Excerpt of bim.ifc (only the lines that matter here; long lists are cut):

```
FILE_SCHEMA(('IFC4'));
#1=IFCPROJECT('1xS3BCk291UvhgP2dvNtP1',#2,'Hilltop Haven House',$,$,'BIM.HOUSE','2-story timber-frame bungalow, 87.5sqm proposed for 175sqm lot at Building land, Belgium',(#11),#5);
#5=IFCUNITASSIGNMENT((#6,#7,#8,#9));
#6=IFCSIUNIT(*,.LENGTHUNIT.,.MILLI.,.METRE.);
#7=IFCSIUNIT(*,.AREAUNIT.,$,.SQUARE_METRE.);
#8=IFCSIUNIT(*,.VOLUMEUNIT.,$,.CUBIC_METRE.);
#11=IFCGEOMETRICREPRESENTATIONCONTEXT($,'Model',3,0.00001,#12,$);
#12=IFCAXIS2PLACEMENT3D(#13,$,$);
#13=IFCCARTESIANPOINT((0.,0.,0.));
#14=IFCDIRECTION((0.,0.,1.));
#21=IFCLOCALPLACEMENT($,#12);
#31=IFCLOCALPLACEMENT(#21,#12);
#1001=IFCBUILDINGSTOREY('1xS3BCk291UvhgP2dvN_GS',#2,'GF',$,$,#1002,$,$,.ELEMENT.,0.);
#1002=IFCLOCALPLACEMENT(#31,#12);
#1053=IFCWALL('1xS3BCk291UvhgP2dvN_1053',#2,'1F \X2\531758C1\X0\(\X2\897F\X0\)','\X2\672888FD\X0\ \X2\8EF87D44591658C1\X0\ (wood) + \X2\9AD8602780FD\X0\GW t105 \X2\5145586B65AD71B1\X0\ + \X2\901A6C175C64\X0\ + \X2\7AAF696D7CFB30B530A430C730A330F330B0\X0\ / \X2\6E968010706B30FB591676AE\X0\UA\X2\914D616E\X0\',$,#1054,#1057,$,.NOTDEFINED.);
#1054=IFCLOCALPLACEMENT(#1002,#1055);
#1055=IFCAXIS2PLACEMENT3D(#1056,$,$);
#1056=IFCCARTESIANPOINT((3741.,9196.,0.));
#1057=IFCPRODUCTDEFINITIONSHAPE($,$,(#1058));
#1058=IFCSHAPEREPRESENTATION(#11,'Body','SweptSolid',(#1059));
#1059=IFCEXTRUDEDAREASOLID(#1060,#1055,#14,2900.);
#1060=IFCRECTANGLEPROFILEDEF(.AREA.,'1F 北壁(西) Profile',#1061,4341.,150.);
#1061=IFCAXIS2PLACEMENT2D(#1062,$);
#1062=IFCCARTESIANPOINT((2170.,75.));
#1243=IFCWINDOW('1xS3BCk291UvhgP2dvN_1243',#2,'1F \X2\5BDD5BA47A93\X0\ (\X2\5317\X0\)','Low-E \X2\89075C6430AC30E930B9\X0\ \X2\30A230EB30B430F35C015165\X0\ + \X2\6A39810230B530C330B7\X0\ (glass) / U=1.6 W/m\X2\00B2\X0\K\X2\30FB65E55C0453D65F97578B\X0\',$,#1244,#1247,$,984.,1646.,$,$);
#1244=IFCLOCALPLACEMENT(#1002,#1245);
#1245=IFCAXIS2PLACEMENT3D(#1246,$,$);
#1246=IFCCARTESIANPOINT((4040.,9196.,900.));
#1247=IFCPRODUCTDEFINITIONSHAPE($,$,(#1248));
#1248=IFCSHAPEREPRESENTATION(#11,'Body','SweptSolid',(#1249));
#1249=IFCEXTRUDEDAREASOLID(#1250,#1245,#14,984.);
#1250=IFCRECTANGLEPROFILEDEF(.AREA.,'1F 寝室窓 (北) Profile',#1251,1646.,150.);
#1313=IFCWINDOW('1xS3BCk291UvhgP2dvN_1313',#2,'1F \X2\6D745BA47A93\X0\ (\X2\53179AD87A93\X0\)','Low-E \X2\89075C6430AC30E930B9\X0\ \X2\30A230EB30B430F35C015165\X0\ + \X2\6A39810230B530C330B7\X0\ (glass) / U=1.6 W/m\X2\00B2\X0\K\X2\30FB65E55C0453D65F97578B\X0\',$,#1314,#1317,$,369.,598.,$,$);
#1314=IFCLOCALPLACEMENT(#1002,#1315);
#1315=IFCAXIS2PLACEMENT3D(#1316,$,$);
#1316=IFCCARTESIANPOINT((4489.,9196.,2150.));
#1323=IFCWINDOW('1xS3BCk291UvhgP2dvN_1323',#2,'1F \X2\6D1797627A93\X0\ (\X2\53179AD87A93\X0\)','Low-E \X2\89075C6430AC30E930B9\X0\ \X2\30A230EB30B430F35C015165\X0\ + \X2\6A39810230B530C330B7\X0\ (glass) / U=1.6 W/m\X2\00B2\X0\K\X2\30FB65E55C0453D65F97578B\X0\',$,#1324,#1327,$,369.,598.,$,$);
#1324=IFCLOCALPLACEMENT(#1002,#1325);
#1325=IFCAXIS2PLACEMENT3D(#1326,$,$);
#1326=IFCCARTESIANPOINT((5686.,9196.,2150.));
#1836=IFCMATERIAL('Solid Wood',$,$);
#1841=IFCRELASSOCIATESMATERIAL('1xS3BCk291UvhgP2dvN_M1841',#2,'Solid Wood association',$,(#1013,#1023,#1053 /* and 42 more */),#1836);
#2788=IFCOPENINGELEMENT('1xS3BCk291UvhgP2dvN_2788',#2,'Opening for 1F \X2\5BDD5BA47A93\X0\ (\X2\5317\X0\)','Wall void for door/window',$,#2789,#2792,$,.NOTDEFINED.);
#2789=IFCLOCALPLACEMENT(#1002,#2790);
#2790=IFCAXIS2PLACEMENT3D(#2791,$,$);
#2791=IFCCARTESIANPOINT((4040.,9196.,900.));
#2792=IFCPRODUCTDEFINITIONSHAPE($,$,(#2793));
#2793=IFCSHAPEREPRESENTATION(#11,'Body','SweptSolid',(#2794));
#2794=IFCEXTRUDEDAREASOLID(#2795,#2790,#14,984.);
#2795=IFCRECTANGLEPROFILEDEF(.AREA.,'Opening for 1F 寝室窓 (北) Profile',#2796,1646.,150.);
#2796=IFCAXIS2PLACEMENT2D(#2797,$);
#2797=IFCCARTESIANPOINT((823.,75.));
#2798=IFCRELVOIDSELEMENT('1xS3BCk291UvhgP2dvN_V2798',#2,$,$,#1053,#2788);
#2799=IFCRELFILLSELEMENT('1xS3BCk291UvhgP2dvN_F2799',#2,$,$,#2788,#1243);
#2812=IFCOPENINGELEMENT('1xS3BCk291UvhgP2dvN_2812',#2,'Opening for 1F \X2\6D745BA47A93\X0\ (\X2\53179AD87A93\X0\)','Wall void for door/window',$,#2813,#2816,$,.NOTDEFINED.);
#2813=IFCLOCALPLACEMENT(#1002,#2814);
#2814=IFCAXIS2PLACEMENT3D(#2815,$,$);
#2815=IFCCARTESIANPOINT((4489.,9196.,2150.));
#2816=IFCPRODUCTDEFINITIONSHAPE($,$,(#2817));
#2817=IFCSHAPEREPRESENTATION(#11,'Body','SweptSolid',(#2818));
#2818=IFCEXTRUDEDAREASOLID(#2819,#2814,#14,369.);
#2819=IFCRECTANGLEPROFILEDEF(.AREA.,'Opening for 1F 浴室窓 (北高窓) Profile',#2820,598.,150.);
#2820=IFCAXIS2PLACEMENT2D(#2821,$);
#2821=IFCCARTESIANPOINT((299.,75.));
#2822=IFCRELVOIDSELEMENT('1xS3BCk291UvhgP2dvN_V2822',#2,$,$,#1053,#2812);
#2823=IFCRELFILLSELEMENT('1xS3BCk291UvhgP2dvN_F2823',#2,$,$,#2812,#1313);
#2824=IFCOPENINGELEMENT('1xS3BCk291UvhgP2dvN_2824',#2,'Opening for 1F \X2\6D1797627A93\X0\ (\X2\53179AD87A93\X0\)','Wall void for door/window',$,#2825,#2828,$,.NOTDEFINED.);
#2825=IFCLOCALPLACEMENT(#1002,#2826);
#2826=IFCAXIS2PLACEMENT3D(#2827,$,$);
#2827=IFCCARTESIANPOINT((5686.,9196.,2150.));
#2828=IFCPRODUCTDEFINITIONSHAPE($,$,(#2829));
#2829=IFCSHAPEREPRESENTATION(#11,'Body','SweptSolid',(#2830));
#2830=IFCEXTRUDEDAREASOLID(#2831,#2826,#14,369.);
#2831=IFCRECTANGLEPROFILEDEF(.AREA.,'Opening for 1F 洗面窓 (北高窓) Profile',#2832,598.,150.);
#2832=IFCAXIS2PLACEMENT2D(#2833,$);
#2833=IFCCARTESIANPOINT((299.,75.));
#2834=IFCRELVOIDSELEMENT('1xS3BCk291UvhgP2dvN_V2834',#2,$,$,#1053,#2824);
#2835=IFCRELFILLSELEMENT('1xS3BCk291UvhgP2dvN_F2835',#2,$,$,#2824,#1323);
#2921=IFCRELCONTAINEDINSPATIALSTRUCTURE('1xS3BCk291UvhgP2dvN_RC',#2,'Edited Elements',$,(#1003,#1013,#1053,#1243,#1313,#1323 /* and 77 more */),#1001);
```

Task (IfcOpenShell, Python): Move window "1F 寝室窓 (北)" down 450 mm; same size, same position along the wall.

```python
import numpy as np
import ifcopenshell
import ifcopenshell.api.geometry
import ifcopenshell.util.placement
import ifcopenshell.util.unit

model = ifcopenshell.open("bim.ifc")
unit_scale = ifcopenshell.util.unit.calculate_unit_scale(model)

window = model.by_guid("1xS3BCk291UvhgP2dvN_1243")
opening = window.FillsVoids[0].RelatingOpeningElement
dz = -450.0

shift = np.array([0.0, 0.0, dz])
# The window is not placed relative to its opening, so move both.
for product in (opening, window):
    matrix = ifcopenshell.util.placement.get_local_placement(product.ObjectPlacement)
    matrix[:3, 3] += shift
    ifcopenshell.api.geometry.edit_object_placement(model, product=product, matrix=matrix, is_si=False)

print(f"moved by {dz * unit_scale:+.3f} m")

model.write("bim_updated.ifc")
```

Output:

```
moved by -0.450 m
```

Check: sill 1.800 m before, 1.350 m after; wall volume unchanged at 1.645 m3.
